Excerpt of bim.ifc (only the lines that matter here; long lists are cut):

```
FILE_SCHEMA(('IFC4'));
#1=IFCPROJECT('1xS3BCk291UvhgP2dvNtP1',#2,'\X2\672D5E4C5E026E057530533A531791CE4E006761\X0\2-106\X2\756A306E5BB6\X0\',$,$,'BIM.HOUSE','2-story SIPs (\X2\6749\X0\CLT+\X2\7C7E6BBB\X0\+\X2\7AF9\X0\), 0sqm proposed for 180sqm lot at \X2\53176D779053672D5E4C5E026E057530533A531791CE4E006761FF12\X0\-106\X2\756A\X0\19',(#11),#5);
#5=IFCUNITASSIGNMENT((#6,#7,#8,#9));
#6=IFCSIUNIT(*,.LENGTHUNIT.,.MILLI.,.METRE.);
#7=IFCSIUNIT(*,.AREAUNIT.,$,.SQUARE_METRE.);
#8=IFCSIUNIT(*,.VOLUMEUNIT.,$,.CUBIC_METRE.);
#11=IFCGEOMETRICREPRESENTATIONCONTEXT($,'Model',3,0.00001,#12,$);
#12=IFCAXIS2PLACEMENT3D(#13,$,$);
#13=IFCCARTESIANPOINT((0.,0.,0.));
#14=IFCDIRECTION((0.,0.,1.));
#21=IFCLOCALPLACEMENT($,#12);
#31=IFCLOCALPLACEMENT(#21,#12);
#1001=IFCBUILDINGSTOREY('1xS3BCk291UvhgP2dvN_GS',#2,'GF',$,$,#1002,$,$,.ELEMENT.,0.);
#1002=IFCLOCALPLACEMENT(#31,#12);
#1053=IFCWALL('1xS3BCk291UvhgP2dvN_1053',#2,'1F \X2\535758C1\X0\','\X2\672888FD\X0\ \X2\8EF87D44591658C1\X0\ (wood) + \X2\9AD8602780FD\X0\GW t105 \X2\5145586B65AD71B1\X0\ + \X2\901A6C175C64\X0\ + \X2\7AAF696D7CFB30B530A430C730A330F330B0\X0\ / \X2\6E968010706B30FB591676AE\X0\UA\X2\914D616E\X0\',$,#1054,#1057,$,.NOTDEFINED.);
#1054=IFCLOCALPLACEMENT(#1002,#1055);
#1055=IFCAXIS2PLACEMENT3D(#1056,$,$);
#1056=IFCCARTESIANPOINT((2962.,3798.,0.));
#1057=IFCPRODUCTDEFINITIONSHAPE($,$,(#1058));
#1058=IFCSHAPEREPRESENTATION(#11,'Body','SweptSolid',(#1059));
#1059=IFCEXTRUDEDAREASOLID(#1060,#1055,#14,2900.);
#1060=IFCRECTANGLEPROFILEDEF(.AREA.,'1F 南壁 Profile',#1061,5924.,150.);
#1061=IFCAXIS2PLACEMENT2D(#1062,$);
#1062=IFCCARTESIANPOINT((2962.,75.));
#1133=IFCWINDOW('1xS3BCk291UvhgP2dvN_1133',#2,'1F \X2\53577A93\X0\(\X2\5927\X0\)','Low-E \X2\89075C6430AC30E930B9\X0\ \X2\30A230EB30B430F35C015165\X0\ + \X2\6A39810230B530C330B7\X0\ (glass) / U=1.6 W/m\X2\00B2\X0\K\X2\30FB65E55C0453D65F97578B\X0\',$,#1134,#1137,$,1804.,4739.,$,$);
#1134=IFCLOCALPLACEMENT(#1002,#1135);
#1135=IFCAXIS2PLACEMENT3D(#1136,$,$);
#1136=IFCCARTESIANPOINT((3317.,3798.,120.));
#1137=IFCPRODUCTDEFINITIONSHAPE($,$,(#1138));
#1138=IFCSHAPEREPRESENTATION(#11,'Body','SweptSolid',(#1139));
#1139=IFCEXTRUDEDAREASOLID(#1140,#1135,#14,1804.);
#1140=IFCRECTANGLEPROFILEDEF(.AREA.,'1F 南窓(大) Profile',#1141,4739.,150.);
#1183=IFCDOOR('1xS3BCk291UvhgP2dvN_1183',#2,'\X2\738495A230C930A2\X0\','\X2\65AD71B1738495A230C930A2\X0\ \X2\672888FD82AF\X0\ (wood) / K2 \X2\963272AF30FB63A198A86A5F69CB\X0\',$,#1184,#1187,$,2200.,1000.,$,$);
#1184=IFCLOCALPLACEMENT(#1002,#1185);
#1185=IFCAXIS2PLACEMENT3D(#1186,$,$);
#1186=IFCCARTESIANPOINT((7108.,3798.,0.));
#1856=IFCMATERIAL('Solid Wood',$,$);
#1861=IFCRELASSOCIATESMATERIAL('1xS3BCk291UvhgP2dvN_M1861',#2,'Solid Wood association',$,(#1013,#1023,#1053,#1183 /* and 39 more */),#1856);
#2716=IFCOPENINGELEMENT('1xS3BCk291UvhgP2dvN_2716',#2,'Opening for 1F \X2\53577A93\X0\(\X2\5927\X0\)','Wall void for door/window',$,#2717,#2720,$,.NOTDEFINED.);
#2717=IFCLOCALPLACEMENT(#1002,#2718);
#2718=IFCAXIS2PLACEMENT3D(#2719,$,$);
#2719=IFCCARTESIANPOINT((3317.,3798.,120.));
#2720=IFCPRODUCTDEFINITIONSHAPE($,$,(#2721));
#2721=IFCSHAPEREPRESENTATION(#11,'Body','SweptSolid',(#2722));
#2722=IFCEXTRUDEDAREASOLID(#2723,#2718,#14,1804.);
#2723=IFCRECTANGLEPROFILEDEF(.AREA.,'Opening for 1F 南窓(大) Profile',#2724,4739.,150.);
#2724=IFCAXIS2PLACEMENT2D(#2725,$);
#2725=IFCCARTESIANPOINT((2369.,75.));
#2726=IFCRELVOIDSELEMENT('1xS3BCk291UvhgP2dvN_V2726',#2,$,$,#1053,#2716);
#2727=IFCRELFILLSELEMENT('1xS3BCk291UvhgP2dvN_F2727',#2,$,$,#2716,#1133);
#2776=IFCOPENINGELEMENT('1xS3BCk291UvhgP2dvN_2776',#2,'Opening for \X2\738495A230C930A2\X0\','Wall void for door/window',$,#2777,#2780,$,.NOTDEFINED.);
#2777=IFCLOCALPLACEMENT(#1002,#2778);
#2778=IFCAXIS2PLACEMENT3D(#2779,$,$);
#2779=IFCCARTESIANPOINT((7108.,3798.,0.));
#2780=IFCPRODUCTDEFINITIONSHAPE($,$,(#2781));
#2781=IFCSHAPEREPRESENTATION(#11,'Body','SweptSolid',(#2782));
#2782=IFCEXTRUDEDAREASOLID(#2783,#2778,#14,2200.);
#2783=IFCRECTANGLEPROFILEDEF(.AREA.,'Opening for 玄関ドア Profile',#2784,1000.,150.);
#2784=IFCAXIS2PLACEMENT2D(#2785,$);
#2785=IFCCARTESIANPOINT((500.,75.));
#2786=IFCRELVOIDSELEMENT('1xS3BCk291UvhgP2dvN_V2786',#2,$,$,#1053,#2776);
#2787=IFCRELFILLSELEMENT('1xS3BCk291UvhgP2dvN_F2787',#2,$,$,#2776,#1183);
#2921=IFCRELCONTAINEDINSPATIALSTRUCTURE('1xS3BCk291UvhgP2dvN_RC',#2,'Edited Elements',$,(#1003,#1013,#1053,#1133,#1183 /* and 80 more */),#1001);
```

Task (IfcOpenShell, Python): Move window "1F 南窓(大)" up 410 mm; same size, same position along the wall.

```python
import numpy as np
import ifcopenshell
import ifcopenshell.api.geometry
import ifcopenshell.util.placement
import ifcopenshell.util.unit

model = ifcopenshell.open("bim.ifc")
unit_scale = ifcopenshell.util.unit.calculate_unit_scale(model)

window = model.by_guid("1xS3BCk291UvhgP2dvN_1133")
opening = window.FillsVoids[0].RelatingOpeningElement
dz = 410.0

shift = np.array([0.0, 0.0, dz])
# The window is not placed relative to its opening, so move both.
for product in (opening, window):
    matrix = ifcopenshell.util.placement.get_local_placement(product.ObjectPlacement)
    matrix[:3, 3] += shift
    ifcopenshell.api.geometry.edit_object_placement(model, product=product, matrix=matrix, is_si=False)

print(f"moved by {dz * unit_scale:+.3f} m")

model.write("bim-out.ifc")
```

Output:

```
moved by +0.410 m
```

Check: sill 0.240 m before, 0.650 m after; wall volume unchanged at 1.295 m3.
